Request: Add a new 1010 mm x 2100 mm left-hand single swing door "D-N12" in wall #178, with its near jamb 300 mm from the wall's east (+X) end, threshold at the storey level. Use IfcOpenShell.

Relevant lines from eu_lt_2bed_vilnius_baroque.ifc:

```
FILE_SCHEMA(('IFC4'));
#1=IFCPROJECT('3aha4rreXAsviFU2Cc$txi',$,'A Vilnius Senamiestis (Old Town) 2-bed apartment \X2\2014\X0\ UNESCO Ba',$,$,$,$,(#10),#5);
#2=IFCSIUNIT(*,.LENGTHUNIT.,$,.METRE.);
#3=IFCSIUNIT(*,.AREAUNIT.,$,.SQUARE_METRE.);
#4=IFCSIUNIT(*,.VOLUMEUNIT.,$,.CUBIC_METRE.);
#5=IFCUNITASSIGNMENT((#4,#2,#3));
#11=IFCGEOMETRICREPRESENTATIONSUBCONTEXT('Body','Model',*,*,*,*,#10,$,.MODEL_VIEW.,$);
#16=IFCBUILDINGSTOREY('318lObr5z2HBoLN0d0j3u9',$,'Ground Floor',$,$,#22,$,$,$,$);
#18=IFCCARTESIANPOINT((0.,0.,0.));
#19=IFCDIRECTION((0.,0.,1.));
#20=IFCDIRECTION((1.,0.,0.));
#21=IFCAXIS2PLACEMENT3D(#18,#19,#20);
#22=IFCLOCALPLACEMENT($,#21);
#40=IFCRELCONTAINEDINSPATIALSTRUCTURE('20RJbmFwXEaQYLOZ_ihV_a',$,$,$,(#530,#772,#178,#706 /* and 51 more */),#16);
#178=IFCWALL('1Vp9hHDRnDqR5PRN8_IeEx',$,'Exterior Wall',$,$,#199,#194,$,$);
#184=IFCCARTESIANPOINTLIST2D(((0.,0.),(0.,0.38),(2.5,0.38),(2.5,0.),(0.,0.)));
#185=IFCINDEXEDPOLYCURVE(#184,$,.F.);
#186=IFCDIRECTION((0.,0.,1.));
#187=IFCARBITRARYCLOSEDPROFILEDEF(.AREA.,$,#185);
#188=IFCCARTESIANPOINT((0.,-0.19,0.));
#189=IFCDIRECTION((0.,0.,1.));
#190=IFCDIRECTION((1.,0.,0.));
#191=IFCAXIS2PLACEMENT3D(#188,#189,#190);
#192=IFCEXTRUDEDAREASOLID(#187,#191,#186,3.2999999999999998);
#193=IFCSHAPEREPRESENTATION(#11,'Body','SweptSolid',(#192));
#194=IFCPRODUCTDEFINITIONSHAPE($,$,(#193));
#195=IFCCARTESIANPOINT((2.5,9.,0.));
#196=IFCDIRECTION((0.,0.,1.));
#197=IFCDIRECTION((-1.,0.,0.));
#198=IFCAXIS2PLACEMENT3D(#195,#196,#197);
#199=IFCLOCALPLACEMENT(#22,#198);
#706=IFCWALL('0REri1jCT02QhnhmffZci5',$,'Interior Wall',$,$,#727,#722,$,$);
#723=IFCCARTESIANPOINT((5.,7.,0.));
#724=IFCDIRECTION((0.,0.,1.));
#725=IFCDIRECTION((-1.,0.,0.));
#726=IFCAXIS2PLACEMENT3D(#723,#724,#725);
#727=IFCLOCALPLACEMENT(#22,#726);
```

```python
import numpy as np
import ifcopenshell
import ifcopenshell.api.feature
import ifcopenshell.api.geometry
import ifcopenshell.api.root
import ifcopenshell.api.spatial
import ifcopenshell.geom
import ifcopenshell.util.element
import ifcopenshell.util.placement
import ifcopenshell.util.representation
import ifcopenshell.util.shape
import ifcopenshell.util.unit

model = ifcopenshell.open("eu_lt_2bed_vilnius_baroque.ifc")
unit_scale = ifcopenshell.util.unit.calculate_unit_scale(model)
settings = ifcopenshell.geom.settings()


def volume(element):
    """Net volume in cubic metres, openings subtracted."""
    shape = ifcopenshell.geom.create_shape(settings, element)
    return ifcopenshell.util.shape.get_volume(shape.geometry)


wall = model.by_guid("1Vp9hHDRnDqR5PRN8_IeEx")
storey = ifcopenshell.util.element.get_container(wall, ifc_class="IfcBuildingStorey")
context = ifcopenshell.util.representation.get_context(model, "Model", "Body", "MODEL_VIEW")
before = volume(wall)

width, height, from_end, sill = 1.01, 2.1, 0.3, 0.0  # metres

# The wall runs along its own X axis, and the end named is its -X end.
wall_shape = ifcopenshell.geom.create_shape(settings, wall)
x, y, z = ifcopenshell.util.shape.get_vertices(wall_shape.geometry).T
start = x.min() + from_end
face, thickness = float(y.min()), float(y.max() - y.min())
wall_matrix = ifcopenshell.util.placement.get_local_placement(wall.ObjectPlacement)
level = ifcopenshell.util.placement.get_local_placement(storey.ObjectPlacement)[2, 3]


def in_wall(x, y):
    """Placement at x, y metres in the wall's axes, at sill height."""
    matrix = wall_matrix.copy()
    matrix[:, 3] = wall_matrix @ np.array([x / unit_scale, y / unit_scale, 0.0, 1.0])
    matrix[2, 3] = level + sill / unit_scale
    return matrix


# Opening: a box that overshoots both wall faces by 50 mm.
opening = ifcopenshell.api.root.create_entity(model, ifc_class="IfcOpeningElement", predefined_type="OPENING")
box = ifcopenshell.api.geometry.add_wall_representation(
    model, context=context, length=width, height=height, thickness=thickness + 0.1
)
ifcopenshell.api.geometry.assign_representation(model, product=opening, representation=box)
ifcopenshell.api.geometry.edit_object_placement(model, product=opening, matrix=in_wall(start, face - 0.05), is_si=False)
ifcopenshell.api.feature.add_feature(model, feature=opening, element=wall)

door = ifcopenshell.api.root.create_entity(model, ifc_class="IfcDoor", name="D-N12", predefined_type="DOOR")
door.OverallWidth, door.OverallHeight = width / unit_scale, height / unit_scale
door.OperationType = "SINGLE_SWING_LEFT"
body = ifcopenshell.api.geometry.add_door_representation(
    model,
    context=context,
    overall_width=door.OverallWidth,
    overall_height=door.OverallHeight,
    operation_type="SINGLE_SWING_LEFT",
    lining_properties={"LiningDepth": thickness / unit_scale, "ThresholdDepth": thickness / unit_scale},
)
ifcopenshell.api.geometry.assign_representation(model, product=door, representation=body)
ifcopenshell.api.spatial.assign_container(model, products=[door], relating_structure=storey)
ifcopenshell.api.feature.add_filling(model, opening=opening, element=door)

# The lining spans the wall, so the door starts at the wall face.
ifcopenshell.api.geometry.edit_object_placement(model, product=door, matrix=in_wall(start, face), is_si=False)

after = volume(wall)

print(f"wall volume {before:.3f} -> {after:.3f} m3")

model.write("eu_lt_2bed_vilnius_baroque_updated.ifc")
```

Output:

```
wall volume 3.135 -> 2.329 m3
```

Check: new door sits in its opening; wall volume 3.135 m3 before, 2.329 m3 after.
